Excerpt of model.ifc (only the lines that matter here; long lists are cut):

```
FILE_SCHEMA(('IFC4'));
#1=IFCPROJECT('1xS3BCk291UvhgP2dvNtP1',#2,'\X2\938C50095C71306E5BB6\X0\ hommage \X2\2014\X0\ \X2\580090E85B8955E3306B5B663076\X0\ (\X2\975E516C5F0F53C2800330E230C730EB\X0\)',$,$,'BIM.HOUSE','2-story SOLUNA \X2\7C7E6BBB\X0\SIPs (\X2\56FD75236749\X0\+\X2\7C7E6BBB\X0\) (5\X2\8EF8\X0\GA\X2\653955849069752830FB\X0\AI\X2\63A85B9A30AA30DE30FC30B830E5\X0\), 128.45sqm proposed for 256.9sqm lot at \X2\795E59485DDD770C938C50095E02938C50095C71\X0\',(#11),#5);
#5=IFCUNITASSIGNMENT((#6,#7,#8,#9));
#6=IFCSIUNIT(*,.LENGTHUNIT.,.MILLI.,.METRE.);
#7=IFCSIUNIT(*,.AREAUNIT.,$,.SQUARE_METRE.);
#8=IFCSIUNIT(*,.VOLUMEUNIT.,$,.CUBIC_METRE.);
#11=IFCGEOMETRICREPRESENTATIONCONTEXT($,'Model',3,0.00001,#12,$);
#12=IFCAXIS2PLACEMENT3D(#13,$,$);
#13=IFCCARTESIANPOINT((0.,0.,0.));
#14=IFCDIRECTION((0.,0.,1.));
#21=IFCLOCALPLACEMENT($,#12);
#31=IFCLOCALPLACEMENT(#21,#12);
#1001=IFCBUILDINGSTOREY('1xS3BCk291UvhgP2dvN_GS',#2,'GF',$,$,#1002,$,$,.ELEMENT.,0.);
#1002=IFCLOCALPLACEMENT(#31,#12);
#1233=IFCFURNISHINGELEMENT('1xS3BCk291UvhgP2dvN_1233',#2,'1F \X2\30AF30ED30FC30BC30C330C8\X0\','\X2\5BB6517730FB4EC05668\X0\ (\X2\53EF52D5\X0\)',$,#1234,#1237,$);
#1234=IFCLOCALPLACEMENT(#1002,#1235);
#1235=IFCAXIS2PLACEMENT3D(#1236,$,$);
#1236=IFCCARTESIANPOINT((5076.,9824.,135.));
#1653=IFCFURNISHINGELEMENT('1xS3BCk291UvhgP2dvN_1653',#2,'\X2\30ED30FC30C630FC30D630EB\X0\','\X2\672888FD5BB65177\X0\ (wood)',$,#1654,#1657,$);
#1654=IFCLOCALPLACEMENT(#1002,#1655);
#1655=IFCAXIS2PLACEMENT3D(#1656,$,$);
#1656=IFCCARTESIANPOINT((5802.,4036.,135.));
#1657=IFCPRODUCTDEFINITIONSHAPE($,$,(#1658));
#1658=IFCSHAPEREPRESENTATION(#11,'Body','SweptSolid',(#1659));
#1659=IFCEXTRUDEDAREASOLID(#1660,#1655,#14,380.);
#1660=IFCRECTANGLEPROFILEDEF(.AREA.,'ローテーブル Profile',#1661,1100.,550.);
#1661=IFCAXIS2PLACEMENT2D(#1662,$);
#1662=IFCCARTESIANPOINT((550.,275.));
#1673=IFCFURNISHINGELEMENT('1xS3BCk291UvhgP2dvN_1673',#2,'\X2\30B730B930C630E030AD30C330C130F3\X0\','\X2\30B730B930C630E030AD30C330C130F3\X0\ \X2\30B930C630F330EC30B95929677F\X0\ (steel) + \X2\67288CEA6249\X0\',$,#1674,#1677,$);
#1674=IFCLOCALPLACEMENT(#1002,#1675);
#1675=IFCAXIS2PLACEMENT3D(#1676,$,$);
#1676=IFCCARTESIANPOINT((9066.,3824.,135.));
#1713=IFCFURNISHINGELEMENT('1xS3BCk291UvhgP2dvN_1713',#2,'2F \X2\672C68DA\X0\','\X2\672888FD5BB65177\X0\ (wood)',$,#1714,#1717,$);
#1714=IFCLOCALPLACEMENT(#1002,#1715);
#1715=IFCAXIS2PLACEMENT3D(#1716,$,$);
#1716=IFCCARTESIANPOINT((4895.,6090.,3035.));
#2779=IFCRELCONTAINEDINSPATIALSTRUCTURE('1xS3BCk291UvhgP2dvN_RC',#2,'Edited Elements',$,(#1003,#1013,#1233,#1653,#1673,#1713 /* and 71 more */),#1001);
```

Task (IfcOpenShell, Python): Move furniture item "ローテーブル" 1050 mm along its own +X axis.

```python
import ifcopenshell
import ifcopenshell.api.geometry
import ifcopenshell.util.placement
import ifcopenshell.util.unit

model = ifcopenshell.open("model.ifc")
unit_scale = ifcopenshell.util.unit.calculate_unit_scale(model)

item = model.by_guid("1xS3BCk291UvhgP2dvN_1653")
matrix = ifcopenshell.util.placement.get_local_placement(item.ObjectPlacement)
matrix[:3, 3] += matrix[:3, 0] * 1.05 / unit_scale
ifcopenshell.api.geometry.edit_object_placement(model, product=item, matrix=matrix, is_si=False)

print(ifcopenshell.util.placement.get_local_placement(item.ObjectPlacement).round(3) + 0.0)

model.write("model_v2.ifc")
```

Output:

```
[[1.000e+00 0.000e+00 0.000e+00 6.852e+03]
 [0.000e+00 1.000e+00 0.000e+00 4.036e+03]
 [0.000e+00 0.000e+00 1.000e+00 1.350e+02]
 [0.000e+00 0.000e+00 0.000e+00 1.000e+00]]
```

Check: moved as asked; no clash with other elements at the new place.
